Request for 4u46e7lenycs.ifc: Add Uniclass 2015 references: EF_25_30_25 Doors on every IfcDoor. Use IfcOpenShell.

First a look at what the model holds.

```python
import ifcopenshell

model = ifcopenshell.open("4u46e7lenycs.ifc")
print(model.schema)
print("classifications:", [c.Name for c in model.by_type("IfcClassification")])
for ifc_class in ("IfcDoor", "IfcRoof", "IfcStair", "IfcWall", "IfcWindow"):
    print(ifc_class, len(model.by_type(ifc_class)))
```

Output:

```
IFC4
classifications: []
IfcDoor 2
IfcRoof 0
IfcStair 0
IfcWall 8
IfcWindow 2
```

```python
import ifcopenshell
import ifcopenshell.api.classification

model = ifcopenshell.open("4u46e7lenycs.ifc")

system = ifcopenshell.api.classification.add_classification(model, classification="Uniclass 2015")

codes = {
    "IfcDoor": ("EF_25_30_25", "Doors"),
}
for ifc_class, (code, name) in codes.items():
    products = model.by_type(ifc_class)
    ifcopenshell.api.classification.add_reference(
        model, products=products, classification=system, identification=code, name=name
    )
    print(code, len(products))

model.write("4u46e7lenycs_v2.ifc")
```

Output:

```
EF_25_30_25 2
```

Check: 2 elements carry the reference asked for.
